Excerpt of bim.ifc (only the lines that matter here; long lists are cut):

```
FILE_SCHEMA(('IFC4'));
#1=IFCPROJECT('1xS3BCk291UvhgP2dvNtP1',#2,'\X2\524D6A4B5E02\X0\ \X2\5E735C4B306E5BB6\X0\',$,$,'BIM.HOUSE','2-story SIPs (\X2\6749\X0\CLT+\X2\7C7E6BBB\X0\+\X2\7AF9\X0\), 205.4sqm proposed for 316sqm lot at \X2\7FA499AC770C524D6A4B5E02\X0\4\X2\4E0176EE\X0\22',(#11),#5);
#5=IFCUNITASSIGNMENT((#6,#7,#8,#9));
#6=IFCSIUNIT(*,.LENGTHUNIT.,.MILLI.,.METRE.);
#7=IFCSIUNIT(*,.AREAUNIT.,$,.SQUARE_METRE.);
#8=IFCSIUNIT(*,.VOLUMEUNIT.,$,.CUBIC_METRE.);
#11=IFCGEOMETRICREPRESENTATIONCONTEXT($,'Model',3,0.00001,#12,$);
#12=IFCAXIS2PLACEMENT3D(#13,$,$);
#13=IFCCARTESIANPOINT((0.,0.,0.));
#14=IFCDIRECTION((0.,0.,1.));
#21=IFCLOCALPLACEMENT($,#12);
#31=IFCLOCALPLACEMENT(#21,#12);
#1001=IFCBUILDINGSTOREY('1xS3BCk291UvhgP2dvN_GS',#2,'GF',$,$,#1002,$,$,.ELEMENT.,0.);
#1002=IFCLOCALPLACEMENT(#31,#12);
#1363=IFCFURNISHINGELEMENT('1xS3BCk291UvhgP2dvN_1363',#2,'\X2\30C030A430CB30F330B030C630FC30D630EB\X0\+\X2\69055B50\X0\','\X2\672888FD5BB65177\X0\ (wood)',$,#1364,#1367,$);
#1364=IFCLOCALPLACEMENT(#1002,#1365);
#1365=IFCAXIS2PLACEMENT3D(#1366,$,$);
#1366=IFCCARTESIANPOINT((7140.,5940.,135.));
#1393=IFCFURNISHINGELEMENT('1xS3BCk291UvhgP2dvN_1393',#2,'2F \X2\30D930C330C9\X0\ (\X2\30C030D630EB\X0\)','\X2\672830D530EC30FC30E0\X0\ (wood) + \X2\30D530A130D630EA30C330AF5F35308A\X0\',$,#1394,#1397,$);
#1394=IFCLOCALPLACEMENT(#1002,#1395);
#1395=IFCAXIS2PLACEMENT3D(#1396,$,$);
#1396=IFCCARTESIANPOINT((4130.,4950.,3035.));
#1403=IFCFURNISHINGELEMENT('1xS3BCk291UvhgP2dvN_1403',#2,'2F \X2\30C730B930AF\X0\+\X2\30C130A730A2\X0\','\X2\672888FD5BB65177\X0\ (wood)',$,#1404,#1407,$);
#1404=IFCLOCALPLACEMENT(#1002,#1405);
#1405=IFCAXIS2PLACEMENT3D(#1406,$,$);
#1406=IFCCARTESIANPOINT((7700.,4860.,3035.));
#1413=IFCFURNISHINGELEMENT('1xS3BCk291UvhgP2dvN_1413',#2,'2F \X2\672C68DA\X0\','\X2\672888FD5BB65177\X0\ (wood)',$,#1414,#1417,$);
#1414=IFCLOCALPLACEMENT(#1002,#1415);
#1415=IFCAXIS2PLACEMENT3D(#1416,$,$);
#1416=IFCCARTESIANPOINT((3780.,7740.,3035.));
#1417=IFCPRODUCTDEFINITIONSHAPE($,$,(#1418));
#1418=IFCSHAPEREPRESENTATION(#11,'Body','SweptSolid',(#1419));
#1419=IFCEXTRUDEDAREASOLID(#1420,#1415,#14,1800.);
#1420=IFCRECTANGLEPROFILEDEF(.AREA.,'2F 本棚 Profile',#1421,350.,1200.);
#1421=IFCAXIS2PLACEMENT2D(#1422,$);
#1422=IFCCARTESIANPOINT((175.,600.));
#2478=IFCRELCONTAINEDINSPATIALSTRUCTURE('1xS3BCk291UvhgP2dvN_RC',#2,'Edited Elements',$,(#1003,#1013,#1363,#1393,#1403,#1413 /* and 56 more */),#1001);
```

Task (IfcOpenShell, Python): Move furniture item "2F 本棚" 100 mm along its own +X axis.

```python
import ifcopenshell
import ifcopenshell.api.geometry
import ifcopenshell.util.placement
import ifcopenshell.util.unit

model = ifcopenshell.open("bim.ifc")
unit_scale = ifcopenshell.util.unit.calculate_unit_scale(model)

item = model.by_guid("1xS3BCk291UvhgP2dvN_1413")
matrix = ifcopenshell.util.placement.get_local_placement(item.ObjectPlacement)
matrix[:3, 3] += matrix[:3, 0] * 0.1 / unit_scale
ifcopenshell.api.geometry.edit_object_placement(model, product=item, matrix=matrix, is_si=False)

print(ifcopenshell.util.placement.get_local_placement(item.ObjectPlacement).round(3) + 0.0)

model.write("bim_rev.ifc")
```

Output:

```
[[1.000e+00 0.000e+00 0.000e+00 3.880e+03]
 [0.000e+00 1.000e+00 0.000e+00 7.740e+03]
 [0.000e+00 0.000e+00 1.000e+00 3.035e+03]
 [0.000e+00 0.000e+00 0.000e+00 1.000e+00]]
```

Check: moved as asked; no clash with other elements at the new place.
